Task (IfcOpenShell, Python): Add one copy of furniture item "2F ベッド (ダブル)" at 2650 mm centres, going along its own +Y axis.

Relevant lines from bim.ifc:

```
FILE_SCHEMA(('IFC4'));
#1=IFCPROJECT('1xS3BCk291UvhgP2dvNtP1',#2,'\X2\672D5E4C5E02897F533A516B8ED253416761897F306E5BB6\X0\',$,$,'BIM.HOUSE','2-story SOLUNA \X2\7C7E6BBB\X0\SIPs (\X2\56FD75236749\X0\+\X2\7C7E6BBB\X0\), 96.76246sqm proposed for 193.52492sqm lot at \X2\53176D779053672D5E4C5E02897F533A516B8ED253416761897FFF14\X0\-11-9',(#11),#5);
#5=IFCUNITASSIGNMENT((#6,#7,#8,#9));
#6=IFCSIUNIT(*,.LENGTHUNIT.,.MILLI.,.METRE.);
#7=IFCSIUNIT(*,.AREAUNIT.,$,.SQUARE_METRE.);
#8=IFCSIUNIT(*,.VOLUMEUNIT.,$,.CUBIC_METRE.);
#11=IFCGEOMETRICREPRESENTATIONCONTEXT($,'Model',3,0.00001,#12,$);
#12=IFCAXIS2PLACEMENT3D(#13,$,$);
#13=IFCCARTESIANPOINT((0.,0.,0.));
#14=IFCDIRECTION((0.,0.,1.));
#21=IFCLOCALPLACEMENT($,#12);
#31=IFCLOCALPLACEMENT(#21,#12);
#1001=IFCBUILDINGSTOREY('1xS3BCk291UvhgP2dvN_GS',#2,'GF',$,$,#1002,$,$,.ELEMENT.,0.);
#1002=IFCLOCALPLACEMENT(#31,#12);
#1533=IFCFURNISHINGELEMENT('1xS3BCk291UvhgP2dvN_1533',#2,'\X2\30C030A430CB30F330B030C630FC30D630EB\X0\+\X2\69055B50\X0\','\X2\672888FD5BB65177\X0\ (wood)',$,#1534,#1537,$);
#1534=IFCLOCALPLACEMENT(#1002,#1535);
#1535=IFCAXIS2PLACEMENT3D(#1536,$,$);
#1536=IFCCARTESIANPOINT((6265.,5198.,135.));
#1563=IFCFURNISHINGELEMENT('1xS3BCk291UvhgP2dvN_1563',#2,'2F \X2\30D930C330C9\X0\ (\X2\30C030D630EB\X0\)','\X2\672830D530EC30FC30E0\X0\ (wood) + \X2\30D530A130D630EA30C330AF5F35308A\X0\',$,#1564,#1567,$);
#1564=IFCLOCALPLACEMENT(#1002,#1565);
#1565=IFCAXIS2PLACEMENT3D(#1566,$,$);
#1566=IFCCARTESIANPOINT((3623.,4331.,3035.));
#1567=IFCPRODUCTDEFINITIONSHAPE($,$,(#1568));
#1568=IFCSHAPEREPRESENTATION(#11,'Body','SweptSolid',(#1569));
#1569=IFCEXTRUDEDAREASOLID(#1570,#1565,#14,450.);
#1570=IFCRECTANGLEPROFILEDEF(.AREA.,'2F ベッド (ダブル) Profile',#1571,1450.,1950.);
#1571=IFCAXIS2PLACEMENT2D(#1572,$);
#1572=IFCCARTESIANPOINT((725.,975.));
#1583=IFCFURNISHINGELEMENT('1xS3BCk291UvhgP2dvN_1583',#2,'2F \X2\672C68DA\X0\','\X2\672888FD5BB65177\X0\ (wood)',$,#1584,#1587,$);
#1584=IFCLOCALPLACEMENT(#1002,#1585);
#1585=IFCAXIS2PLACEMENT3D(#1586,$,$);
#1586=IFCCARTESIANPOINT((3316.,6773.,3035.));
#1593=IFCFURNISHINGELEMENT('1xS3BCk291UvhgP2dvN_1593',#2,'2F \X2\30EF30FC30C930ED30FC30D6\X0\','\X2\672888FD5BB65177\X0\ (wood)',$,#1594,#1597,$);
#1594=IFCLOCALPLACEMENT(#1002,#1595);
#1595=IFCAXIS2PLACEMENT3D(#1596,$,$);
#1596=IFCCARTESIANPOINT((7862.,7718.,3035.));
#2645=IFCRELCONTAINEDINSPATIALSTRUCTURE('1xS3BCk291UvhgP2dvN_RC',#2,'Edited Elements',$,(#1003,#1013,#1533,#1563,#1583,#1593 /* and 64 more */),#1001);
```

```python
import ifcopenshell
import ifcopenshell.api.geometry
import ifcopenshell.api.root
import ifcopenshell.util.element
import ifcopenshell.util.placement
import ifcopenshell.util.unit

model = ifcopenshell.open("bim.ifc")
unit_scale = ifcopenshell.util.unit.calculate_unit_scale(model)


def reuse_history(source, copy):
    """copy_class also copies each property set's owner history, people and application; keep the originals."""
    for rel in copy.IsDefinedBy:
        if rel.is_a("IfcRelDefinesByProperties") and (history := rel.RelatingPropertyDefinition.OwnerHistory):
            rel.RelatingPropertyDefinition.OwnerHistory = source.OwnerHistory
            ifcopenshell.util.element.remove_deep2(model, history)


source = model.by_id(1563)
base = ifcopenshell.util.placement.get_local_placement(source.ObjectPlacement)
step = base[:3, 1] * 2.65 / unit_scale

for i in range(1, 2):
    copy = ifcopenshell.api.root.copy_class(model, product=source)
    copy.Representation = ifcopenshell.util.element.copy_deep(
        model, source.Representation, exclude=["IfcGeometricRepresentationContext", "IfcRepresentationMap"]
    )
    reuse_history(source, copy)
    matrix = base.copy()
    matrix[:3, 3] += i * step
    print("added at", matrix[:3, 3].round(3) + 0.0)
    ifcopenshell.api.geometry.edit_object_placement(model, product=copy, matrix=matrix, is_si=False)

model.write("bim_edited.ifc")
```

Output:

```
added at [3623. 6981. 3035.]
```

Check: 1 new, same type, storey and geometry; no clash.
